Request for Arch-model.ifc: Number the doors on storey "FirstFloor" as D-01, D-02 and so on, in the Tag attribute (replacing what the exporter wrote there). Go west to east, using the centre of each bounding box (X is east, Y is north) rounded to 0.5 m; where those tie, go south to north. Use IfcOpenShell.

First a look at what the model holds.

```python
import ifcopenshell
import ifcopenshell.util.element
import ifcopenshell.util.placement

model = ifcopenshell.open("Arch-model.ifc")
print(model.schema)
storey = next(s for s in model.by_type("IfcBuildingStorey") if s.Name == "FirstFloor")
doors = [e for e in ifcopenshell.util.element.get_decomposition(storey) if e.is_a("IfcDoor")]
for e in sorted(doors, key=lambda e: e.id()):
    origin = ifcopenshell.util.placement.get_local_placement(e.ObjectPlacement)[:3, 3]
    print(e.id(), e.Tag, e.Name, origin.round(2) + 0.0, sep=" | ")
```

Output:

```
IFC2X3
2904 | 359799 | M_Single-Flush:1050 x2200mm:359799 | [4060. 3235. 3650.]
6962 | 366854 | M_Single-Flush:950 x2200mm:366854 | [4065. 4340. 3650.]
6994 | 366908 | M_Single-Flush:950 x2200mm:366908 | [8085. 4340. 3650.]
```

```python
import ifcopenshell
import ifcopenshell.geom
import ifcopenshell.util.element
import ifcopenshell.util.shape

model = ifcopenshell.open("Arch-model.ifc")
settings = ifcopenshell.geom.settings()
settings.set("use-world-coords", True)


def centre(element):
    shape = ifcopenshell.geom.create_shape(settings, element)
    return ifcopenshell.util.shape.get_bbox_centroid(shape.geometry)


storey = next(s for s in model.by_type("IfcBuildingStorey") if s.Name == "FirstFloor")
doors = [e for e in ifcopenshell.util.element.get_decomposition(storey) if e.is_a("IfcDoor")]

# Insertion points can sit at a corner or the storey origin, so sort by the geometry (in metres).
centres = {e: centre(e) for e in doors}
doors.sort(key=lambda e: (round(centres[e][0] / 0.5), centres[e][1]))

for i, e in enumerate(doors, start=1):
    number = f"D-{i:02d}"
    e.Tag = number
    print(e.id(), number)

model.write("Arch-model_updated.ifc")
```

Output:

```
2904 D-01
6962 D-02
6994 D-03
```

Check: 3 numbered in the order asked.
